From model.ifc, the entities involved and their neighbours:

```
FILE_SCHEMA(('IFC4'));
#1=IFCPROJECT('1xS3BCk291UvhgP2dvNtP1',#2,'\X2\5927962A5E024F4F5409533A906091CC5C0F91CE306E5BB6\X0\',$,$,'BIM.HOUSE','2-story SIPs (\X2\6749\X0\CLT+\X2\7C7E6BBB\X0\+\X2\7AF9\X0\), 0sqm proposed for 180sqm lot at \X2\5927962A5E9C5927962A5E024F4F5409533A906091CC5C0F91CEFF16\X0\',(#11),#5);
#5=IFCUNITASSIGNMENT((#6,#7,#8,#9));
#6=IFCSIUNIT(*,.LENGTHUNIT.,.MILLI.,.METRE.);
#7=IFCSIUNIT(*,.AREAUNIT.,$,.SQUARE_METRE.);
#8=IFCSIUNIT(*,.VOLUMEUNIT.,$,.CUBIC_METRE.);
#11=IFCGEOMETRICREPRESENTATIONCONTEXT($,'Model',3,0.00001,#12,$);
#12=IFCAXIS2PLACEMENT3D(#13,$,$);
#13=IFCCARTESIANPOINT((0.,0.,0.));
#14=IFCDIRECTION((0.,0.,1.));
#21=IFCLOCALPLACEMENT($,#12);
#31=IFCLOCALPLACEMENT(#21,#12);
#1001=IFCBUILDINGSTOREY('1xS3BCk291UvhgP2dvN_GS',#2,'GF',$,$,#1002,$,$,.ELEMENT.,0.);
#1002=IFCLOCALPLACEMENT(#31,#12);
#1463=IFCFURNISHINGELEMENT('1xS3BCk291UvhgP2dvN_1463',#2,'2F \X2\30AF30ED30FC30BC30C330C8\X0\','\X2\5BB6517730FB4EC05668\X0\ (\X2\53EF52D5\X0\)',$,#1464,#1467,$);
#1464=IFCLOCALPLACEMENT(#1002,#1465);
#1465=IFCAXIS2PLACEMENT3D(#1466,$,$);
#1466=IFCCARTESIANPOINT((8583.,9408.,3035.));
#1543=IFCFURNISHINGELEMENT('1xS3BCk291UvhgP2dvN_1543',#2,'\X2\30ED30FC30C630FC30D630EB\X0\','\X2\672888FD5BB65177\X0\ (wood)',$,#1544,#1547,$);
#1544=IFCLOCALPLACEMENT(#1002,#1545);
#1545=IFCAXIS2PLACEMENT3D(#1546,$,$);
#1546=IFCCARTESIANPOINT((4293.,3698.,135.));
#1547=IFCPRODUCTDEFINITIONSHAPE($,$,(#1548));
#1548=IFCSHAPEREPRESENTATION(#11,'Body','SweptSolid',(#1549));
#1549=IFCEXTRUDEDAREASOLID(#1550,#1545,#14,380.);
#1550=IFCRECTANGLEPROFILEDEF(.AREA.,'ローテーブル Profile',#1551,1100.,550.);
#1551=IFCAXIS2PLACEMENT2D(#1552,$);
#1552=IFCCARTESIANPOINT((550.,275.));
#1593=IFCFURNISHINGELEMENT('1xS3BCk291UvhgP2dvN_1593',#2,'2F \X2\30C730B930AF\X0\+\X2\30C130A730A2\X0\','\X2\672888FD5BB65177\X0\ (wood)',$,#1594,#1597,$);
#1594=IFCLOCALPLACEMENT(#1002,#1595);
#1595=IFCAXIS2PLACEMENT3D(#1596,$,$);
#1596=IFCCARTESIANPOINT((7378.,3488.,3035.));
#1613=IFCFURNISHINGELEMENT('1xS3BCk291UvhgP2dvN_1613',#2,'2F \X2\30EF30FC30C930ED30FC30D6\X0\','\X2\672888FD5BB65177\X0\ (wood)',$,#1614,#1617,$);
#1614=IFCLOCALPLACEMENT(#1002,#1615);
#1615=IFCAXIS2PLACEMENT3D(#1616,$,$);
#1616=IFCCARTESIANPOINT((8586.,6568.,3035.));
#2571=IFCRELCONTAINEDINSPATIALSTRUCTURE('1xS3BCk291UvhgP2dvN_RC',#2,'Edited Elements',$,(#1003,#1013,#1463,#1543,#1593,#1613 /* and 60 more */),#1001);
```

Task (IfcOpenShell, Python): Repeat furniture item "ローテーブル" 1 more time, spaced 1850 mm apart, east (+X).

```python
import numpy as np
import ifcopenshell
import ifcopenshell.api.geometry
import ifcopenshell.api.root
import ifcopenshell.util.element
import ifcopenshell.util.placement
import ifcopenshell.util.unit

model = ifcopenshell.open("model.ifc")
unit_scale = ifcopenshell.util.unit.calculate_unit_scale(model)


def reuse_history(source, copy):
    """copy_class also copies each property set's owner history, people and application; keep the originals."""
    for rel in copy.IsDefinedBy:
        if rel.is_a("IfcRelDefinesByProperties") and (history := rel.RelatingPropertyDefinition.OwnerHistory):
            rel.RelatingPropertyDefinition.OwnerHistory = source.OwnerHistory
            ifcopenshell.util.element.remove_deep2(model, history)


source = model.by_id(1543)
base = ifcopenshell.util.placement.get_local_placement(source.ObjectPlacement)
step = np.array([1.0, 0.0, 0.0]) * 1.85 / unit_scale

for i in range(1, 2):
    copy = ifcopenshell.api.root.copy_class(model, product=source)
    copy.Representation = ifcopenshell.util.element.copy_deep(
        model, source.Representation, exclude=["IfcGeometricRepresentationContext", "IfcRepresentationMap"]
    )
    reuse_history(source, copy)
    matrix = base.copy()
    matrix[:3, 3] += i * step
    print("added at", matrix[:3, 3].round(3) + 0.0)
    ifcopenshell.api.geometry.edit_object_placement(model, product=copy, matrix=matrix, is_si=False)

model.write("model_rev.ifc")
```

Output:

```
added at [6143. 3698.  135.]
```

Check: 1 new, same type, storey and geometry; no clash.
